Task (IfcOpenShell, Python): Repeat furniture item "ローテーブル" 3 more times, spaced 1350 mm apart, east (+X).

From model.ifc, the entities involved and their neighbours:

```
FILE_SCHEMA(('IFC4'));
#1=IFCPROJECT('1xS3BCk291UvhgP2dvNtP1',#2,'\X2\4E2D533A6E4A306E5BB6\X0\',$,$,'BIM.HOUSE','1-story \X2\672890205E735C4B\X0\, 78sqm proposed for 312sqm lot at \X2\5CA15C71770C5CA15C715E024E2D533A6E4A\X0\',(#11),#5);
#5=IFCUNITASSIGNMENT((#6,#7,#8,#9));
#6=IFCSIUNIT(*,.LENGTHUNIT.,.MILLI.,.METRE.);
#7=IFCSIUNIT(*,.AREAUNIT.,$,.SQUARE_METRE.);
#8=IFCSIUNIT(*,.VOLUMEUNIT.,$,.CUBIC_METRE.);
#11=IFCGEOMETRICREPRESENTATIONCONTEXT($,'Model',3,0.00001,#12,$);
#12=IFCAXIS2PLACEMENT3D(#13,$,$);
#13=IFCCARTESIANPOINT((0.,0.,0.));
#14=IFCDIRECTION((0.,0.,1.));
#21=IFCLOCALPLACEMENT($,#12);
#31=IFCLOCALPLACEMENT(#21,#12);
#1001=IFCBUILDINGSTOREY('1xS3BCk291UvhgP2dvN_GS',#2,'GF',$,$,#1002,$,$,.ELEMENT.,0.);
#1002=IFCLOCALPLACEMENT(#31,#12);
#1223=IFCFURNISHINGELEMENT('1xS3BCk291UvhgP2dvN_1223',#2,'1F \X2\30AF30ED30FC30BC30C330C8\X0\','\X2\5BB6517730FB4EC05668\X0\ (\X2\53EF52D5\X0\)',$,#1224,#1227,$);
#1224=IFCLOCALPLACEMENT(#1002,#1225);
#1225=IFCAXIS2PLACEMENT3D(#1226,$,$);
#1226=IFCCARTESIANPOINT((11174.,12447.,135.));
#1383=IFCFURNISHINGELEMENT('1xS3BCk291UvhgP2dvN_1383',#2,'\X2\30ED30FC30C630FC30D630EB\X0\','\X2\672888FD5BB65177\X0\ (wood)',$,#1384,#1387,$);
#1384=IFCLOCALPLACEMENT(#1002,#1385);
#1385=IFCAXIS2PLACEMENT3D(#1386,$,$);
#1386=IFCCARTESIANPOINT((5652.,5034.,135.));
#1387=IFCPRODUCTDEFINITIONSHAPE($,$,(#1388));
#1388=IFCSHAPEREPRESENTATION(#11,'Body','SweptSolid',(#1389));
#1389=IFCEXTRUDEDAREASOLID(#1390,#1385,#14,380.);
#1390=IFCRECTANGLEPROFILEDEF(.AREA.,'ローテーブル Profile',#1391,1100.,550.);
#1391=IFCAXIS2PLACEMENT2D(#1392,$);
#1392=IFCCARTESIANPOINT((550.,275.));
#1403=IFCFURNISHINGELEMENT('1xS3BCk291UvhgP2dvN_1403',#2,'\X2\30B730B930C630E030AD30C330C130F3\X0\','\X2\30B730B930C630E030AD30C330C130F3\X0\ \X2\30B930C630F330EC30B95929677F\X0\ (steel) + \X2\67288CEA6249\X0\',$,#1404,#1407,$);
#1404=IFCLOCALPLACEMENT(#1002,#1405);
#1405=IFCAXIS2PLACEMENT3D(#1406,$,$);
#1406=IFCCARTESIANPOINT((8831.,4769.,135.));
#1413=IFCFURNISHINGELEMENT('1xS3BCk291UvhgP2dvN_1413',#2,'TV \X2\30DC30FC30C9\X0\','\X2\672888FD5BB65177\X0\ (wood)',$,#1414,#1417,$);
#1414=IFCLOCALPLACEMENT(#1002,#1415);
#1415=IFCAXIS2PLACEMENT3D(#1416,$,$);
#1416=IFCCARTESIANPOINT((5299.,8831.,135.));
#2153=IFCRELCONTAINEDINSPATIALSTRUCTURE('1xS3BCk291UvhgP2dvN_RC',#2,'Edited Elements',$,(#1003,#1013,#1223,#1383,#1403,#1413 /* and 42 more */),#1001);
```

```python
import numpy as np
import ifcopenshell
import ifcopenshell.api.geometry
import ifcopenshell.api.root
import ifcopenshell.util.element
import ifcopenshell.util.placement

model = ifcopenshell.open("model.ifc")


def reuse_history(source, copy):
    """copy_class also copies each property set's owner history, people and application; keep the originals."""
    for rel in copy.IsDefinedBy:
        if rel.is_a("IfcRelDefinesByProperties") and (history := rel.RelatingPropertyDefinition.OwnerHistory):
            rel.RelatingPropertyDefinition.OwnerHistory = source.OwnerHistory
            ifcopenshell.util.element.remove_deep2(model, history)


source = model.by_guid("1xS3BCk291UvhgP2dvN_1383")
base = ifcopenshell.util.placement.get_local_placement(source.ObjectPlacement)
step = np.array([1.0, 0.0, 0.0]) * 1350.0

for i in range(1, 4):
    copy = ifcopenshell.api.root.copy_class(model, product=source)
    copy.Representation = ifcopenshell.util.element.copy_deep(
        model, source.Representation, exclude=["IfcGeometricRepresentationContext", "IfcRepresentationMap"]
    )
    reuse_history(source, copy)
    matrix = base.copy()
    matrix[:3, 3] += i * step
    print("added at", matrix[:3, 3].round(3) + 0.0)
    ifcopenshell.api.geometry.edit_object_placement(model, product=copy, matrix=matrix, is_si=False)

model.write("model_edited.ifc")
```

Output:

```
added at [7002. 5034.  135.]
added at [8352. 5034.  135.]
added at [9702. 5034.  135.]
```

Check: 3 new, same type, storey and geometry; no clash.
